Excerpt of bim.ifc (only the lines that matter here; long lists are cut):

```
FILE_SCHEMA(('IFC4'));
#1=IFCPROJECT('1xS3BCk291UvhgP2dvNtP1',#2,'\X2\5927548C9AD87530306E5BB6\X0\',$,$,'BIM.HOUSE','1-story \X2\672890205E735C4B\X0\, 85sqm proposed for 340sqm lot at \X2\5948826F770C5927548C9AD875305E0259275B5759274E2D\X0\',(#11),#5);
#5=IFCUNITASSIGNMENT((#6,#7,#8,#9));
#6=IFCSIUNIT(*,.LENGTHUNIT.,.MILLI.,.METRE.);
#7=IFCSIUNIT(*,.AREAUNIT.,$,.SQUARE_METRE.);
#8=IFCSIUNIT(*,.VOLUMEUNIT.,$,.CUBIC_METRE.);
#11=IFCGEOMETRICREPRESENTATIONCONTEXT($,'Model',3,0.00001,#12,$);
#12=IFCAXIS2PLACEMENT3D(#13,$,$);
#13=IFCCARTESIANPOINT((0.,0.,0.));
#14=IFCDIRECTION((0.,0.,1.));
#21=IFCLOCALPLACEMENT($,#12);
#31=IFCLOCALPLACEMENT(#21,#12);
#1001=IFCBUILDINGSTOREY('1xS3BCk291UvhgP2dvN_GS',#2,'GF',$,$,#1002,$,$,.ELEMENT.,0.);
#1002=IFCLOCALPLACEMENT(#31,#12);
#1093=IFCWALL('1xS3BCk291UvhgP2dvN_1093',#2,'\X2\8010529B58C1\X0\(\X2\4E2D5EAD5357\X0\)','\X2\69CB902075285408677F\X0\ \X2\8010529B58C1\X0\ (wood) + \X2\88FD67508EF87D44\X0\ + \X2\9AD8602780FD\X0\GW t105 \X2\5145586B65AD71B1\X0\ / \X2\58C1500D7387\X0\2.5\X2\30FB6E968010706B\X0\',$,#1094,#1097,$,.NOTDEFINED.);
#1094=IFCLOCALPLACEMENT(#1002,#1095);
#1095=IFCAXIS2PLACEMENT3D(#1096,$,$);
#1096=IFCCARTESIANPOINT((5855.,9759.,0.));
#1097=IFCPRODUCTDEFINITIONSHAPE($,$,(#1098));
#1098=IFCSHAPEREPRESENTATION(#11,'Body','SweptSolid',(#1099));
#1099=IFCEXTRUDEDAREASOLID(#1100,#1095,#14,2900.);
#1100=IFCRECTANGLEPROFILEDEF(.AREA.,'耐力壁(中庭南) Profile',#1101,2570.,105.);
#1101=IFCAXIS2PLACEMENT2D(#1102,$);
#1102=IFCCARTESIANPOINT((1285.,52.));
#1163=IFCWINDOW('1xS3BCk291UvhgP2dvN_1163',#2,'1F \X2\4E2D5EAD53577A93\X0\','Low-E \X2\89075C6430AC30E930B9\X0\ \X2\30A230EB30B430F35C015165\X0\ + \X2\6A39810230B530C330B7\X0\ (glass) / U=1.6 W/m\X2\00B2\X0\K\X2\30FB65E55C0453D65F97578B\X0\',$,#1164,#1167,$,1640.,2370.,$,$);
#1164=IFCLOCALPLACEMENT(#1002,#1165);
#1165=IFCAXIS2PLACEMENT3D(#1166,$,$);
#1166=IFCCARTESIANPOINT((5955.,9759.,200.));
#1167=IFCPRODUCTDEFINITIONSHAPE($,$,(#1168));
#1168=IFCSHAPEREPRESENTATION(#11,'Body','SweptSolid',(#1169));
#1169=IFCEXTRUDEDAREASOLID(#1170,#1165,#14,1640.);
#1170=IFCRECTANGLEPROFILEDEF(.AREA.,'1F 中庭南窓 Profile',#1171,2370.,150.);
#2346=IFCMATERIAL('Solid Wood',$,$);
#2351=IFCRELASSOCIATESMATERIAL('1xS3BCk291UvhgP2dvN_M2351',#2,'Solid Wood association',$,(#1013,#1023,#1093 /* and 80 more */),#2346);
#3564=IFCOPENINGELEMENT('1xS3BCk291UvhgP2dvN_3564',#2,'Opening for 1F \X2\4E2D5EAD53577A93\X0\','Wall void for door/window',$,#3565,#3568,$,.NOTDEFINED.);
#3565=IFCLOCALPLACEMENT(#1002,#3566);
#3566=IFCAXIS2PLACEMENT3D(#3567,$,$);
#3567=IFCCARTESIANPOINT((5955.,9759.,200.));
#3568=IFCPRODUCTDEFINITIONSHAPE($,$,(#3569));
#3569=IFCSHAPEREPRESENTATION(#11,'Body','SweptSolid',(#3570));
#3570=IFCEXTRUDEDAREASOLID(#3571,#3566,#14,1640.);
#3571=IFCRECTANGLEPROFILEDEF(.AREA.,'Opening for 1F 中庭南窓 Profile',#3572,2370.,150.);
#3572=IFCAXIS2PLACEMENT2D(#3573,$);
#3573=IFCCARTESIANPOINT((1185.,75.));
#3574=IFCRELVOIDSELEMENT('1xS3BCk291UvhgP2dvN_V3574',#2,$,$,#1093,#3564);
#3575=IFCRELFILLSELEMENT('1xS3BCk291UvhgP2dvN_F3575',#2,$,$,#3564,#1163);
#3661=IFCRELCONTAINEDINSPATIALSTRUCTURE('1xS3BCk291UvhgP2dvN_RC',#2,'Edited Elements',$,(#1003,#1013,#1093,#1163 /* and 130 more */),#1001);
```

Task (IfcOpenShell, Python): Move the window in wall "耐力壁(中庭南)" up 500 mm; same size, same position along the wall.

```python
import numpy as np
import ifcopenshell
import ifcopenshell.api.geometry
import ifcopenshell.util.placement
import ifcopenshell.util.unit

model = ifcopenshell.open("bim.ifc")
unit_scale = ifcopenshell.util.unit.calculate_unit_scale(model)

window = model.by_guid("1xS3BCk291UvhgP2dvN_1163")
opening = window.FillsVoids[0].RelatingOpeningElement
dz = 500.0

shift = np.array([0.0, 0.0, dz])
# The window is not placed relative to its opening, so move both.
for product in (opening, window):
    matrix = ifcopenshell.util.placement.get_local_placement(product.ObjectPlacement)
    matrix[:3, 3] += shift
    ifcopenshell.api.geometry.edit_object_placement(model, product=product, matrix=matrix, is_si=False)

print(f"moved by {dz * unit_scale:+.3f} m")

model.write("bim_edited.ifc")
```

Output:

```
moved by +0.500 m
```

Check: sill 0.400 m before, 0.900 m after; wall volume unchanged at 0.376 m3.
